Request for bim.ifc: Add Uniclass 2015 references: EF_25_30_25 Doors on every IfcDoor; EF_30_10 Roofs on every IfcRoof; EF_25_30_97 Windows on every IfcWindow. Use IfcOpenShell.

First a look at what the model holds.

```python
import ifcopenshell

model = ifcopenshell.open("bim.ifc")
print(model.schema)
print("classifications:", [c.Name for c in model.by_type("IfcClassification")])
for ifc_class in ("IfcDoor", "IfcRoof", "IfcStair", "IfcWall", "IfcWindow"):
    print(ifc_class, len(model.by_type(ifc_class)))
```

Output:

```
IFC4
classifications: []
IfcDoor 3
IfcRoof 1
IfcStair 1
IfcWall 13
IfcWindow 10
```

```python
import ifcopenshell
import ifcopenshell.api.classification

model = ifcopenshell.open("bim.ifc")

system = ifcopenshell.api.classification.add_classification(model, classification="Uniclass 2015")

codes = {
    "IfcDoor": ("EF_25_30_25", "Doors"),
    "IfcRoof": ("EF_30_10", "Roofs"),
    "IfcWindow": ("EF_25_30_97", "Windows"),
}
for ifc_class, (code, name) in codes.items():
    products = model.by_type(ifc_class)
    ifcopenshell.api.classification.add_reference(
        model, products=products, classification=system, identification=code, name=name
    )
    print(code, len(products))

model.write("bim_v2.ifc")
```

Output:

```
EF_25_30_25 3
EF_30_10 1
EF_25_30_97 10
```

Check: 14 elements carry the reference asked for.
